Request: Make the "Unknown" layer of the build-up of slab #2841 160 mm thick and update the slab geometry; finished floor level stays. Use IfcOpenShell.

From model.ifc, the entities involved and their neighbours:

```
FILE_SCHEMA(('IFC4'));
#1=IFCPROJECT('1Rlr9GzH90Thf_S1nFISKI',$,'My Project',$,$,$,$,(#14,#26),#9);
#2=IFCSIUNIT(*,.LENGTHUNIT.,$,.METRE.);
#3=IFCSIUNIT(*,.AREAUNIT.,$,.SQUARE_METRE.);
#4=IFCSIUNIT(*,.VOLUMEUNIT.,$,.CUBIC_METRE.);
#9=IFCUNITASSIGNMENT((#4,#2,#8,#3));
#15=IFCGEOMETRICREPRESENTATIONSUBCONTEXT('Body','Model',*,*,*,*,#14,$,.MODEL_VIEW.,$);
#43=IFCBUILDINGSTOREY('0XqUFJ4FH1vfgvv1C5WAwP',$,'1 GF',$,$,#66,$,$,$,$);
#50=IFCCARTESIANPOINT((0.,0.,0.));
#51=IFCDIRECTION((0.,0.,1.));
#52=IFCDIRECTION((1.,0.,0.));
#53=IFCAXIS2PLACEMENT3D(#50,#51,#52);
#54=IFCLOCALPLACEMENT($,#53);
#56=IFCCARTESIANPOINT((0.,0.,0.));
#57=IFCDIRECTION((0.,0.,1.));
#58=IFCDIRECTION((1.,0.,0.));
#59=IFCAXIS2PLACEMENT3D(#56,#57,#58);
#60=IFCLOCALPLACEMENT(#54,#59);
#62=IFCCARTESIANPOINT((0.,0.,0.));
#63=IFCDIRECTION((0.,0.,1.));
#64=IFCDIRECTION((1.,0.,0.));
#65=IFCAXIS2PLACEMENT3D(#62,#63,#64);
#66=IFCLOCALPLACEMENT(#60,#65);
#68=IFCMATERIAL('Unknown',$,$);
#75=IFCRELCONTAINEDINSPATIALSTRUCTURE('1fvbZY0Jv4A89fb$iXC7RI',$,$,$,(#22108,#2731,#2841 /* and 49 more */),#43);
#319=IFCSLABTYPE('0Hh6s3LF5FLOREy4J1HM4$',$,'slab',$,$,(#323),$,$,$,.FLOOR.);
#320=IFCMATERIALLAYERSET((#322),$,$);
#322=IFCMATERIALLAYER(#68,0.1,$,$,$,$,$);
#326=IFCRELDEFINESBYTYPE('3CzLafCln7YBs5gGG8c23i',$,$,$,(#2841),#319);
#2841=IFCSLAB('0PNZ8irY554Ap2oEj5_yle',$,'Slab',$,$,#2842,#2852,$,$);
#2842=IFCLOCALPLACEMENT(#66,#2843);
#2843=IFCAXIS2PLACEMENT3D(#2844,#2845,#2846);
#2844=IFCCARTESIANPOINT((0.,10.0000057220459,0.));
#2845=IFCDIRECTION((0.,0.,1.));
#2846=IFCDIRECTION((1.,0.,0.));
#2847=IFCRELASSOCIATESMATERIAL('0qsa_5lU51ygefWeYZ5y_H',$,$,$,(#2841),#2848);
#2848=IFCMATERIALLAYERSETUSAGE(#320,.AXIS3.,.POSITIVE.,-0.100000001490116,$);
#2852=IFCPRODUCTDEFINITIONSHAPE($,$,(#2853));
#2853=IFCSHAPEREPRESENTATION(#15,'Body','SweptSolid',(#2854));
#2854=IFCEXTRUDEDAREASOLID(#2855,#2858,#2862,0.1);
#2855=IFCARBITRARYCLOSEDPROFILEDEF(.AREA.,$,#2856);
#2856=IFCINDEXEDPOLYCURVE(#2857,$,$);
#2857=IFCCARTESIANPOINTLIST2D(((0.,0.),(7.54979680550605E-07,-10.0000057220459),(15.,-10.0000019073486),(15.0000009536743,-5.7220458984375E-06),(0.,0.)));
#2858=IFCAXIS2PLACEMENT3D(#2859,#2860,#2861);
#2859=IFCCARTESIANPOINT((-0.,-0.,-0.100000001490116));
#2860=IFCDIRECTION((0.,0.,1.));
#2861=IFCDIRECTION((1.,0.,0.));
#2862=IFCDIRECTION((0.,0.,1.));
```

```python
import ifcopenshell
import ifcopenshell.util.element
import ifcopenshell.util.representation
import ifcopenshell.util.unit

model = ifcopenshell.open("model.ifc")
unit_scale = ifcopenshell.util.unit.calculate_unit_scale(model)

layer_set = model.by_id(320)
layer = next(l for l in layer_set.MaterialLayers if l.Material and l.Material.Name == "Unknown")
change = 0.16 / unit_scale - layer.LayerThickness
layer.LayerThickness += change

# Geometry does not follow the layer set by itself.
slabs = [e for e in ifcopenshell.util.element.get_elements_by_material(model, layer_set) if e.is_a("IfcSlab")]
for slab in sorted(slabs, key=lambda e: e.id()):
    body = ifcopenshell.util.representation.get_representation(slab, "Model", "Body")
    solid = body.Items[0]
    old_depth = solid.Depth
    solid.Depth += change
    # Extruded upwards: lower the start of the extrusion so the top stays.
    x, y, z = solid.Position.Location.Coordinates
    solid.Position.Location = model.createIfcCartesianPoint((x, y, z - change))
    print(slab.id(), f"{old_depth:g} -> {solid.Depth:g}")

# The layers are counted up from the underside, which has moved.
for usage in {ifcopenshell.util.element.get_material(slab) for slab in slabs}:
    usage.OffsetFromReferenceLine -= change

model.write("model-out.ifc")
```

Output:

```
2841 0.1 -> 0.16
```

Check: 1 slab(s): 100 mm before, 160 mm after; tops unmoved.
